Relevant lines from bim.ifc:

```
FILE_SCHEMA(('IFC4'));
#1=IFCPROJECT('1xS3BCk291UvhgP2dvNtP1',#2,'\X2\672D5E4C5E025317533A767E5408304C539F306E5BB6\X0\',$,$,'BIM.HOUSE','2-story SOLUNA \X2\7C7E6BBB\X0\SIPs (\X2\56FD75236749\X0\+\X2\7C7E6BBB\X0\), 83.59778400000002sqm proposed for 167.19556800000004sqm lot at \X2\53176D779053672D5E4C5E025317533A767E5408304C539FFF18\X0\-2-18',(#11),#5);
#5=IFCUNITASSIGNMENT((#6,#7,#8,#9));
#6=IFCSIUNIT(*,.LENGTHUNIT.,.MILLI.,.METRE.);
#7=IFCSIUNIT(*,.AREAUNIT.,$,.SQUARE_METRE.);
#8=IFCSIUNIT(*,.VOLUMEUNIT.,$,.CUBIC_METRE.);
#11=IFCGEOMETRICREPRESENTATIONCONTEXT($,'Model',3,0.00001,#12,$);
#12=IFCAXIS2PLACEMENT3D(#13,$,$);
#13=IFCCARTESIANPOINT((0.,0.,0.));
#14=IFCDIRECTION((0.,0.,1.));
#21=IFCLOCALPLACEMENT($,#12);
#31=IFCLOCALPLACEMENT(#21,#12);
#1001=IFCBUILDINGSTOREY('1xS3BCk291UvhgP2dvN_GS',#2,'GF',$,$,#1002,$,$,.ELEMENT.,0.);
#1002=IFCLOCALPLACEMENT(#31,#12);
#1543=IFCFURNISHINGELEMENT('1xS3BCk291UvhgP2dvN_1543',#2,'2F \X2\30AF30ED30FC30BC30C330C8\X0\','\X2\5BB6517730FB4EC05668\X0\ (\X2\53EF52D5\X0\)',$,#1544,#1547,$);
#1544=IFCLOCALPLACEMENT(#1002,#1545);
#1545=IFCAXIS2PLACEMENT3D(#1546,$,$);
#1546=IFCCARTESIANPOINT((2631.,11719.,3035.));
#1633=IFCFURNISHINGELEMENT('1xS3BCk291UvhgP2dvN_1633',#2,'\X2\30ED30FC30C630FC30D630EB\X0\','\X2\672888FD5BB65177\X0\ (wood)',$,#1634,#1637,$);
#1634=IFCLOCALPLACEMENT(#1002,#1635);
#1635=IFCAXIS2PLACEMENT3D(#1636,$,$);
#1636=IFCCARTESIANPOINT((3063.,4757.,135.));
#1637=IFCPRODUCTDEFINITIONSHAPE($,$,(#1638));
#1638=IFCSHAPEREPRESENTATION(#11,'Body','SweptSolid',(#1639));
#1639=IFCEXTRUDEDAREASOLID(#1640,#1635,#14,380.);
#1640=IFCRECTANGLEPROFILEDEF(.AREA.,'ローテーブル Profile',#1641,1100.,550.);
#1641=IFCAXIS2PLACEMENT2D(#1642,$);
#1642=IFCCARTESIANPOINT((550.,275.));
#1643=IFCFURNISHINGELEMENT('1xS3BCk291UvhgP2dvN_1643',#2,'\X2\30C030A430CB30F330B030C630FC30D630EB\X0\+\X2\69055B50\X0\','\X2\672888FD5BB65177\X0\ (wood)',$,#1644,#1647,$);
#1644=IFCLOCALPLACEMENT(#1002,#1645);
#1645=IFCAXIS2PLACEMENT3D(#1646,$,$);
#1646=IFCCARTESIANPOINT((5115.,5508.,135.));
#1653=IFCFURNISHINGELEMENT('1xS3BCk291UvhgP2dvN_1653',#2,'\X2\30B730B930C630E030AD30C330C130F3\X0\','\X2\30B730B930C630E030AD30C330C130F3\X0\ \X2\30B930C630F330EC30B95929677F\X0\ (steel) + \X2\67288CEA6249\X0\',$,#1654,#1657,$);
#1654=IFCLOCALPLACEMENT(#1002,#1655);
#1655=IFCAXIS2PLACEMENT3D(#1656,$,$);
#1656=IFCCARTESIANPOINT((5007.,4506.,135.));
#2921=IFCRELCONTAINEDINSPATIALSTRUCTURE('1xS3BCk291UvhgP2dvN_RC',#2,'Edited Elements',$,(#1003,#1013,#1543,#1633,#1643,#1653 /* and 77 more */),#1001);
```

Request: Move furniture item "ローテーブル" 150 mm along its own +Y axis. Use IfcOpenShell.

```python
import ifcopenshell
import ifcopenshell.api.geometry
import ifcopenshell.util.placement
import ifcopenshell.util.unit

model = ifcopenshell.open("bim.ifc")
unit_scale = ifcopenshell.util.unit.calculate_unit_scale(model)

item = model.by_id(1633)
matrix = ifcopenshell.util.placement.get_local_placement(item.ObjectPlacement)
matrix[:3, 3] += matrix[:3, 1] * 0.15 / unit_scale
ifcopenshell.api.geometry.edit_object_placement(model, product=item, matrix=matrix, is_si=False)

print(ifcopenshell.util.placement.get_local_placement(item.ObjectPlacement).round(3) + 0.0)

model.write("bim_edited.ifc")
```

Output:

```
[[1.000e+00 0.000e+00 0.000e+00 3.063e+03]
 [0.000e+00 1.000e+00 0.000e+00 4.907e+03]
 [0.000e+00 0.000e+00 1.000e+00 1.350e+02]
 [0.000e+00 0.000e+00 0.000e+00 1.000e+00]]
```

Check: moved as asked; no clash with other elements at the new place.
